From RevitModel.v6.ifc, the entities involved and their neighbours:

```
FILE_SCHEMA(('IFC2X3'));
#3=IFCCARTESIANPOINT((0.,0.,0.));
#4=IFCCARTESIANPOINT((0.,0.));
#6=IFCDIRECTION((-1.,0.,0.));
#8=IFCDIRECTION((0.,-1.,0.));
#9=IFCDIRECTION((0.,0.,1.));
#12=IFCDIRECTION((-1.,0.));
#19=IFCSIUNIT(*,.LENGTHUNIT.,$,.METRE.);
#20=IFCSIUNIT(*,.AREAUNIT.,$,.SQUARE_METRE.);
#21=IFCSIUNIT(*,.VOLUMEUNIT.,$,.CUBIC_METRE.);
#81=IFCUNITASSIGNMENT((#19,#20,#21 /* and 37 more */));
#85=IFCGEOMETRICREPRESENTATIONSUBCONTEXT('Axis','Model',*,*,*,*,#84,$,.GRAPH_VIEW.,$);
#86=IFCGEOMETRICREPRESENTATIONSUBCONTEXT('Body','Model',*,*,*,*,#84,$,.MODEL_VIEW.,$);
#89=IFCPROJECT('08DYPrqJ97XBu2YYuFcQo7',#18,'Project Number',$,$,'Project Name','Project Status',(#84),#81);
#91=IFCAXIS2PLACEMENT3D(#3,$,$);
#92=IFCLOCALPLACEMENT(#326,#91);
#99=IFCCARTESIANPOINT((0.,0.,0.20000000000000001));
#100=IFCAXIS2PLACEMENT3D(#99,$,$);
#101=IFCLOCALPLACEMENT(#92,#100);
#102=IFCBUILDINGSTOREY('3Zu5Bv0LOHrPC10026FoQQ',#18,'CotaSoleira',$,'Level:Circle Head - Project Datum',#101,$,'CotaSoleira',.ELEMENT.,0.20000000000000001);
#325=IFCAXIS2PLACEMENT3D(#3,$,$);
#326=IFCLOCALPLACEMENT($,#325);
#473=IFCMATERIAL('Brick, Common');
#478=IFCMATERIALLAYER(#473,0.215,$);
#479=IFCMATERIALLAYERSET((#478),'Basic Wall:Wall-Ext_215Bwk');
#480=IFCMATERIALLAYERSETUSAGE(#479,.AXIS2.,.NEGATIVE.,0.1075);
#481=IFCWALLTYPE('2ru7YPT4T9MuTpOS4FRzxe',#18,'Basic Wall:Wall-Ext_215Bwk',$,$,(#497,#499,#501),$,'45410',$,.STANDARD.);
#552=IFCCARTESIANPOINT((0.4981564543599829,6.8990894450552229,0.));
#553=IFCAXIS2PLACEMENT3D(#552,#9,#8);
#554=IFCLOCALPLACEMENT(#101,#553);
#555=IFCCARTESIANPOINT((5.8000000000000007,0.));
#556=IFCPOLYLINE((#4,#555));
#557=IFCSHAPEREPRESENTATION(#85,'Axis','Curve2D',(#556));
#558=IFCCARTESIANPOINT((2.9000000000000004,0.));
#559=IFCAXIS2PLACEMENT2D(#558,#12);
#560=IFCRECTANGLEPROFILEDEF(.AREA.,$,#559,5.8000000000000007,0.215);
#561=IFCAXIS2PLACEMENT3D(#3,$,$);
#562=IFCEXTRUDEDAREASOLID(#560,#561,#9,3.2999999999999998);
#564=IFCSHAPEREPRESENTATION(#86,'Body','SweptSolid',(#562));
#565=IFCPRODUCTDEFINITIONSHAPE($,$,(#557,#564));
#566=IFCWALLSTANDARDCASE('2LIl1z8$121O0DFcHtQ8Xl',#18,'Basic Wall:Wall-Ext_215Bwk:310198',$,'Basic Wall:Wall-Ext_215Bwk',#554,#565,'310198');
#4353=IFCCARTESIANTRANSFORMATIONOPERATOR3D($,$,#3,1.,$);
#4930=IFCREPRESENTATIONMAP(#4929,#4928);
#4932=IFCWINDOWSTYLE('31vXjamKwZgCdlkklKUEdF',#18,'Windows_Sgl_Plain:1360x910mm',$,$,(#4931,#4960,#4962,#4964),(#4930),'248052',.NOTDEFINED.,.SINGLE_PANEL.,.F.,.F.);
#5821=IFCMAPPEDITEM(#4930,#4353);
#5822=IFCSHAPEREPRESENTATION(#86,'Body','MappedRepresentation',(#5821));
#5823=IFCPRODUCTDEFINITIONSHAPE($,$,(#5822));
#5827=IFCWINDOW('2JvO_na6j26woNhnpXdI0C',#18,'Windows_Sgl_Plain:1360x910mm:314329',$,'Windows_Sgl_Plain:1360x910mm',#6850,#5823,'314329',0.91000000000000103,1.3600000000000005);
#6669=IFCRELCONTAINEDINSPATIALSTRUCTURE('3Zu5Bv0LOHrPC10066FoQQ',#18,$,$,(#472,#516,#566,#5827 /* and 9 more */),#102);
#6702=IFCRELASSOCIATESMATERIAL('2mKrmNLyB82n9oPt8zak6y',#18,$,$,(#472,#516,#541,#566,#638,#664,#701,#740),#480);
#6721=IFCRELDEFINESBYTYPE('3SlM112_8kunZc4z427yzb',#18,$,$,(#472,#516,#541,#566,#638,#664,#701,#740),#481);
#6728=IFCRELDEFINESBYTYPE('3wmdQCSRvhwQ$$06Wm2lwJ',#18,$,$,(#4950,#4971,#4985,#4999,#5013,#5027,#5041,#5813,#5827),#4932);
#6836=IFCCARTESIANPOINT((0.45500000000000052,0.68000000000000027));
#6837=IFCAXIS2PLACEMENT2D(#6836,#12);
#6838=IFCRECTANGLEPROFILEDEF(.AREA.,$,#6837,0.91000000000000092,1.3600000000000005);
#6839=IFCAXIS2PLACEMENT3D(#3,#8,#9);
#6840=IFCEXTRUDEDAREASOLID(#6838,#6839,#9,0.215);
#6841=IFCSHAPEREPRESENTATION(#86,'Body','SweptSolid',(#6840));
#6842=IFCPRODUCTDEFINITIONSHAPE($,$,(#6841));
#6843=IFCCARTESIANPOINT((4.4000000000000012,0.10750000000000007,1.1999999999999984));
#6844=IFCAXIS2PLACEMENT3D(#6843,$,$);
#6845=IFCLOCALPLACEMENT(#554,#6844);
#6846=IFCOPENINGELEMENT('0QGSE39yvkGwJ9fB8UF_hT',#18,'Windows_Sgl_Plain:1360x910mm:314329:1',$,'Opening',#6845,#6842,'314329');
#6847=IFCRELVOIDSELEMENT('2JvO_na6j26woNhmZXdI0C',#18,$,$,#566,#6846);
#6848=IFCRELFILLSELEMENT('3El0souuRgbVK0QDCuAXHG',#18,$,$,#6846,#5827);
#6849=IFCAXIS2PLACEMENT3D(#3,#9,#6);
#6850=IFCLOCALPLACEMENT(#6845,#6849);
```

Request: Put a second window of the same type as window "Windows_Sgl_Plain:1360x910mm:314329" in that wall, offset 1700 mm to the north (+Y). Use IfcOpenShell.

```python
import ifcopenshell
import ifcopenshell.api.feature
import ifcopenshell.api.geometry
import ifcopenshell.api.root
import ifcopenshell.geom
import ifcopenshell.util.element
import ifcopenshell.util.placement
import ifcopenshell.util.shape

model = ifcopenshell.open("RevitModel.v6.ifc")
settings = ifcopenshell.geom.settings()


def volume(element):
    """Net volume in cubic metres, openings subtracted."""
    shape = ifcopenshell.geom.create_shape(settings, element)
    return ifcopenshell.util.shape.get_volume(shape.geometry)


def reuse_history(source, copy):
    """copy_class also copies each property set's owner history, people and application; keep the originals."""
    for rel in copy.IsDefinedBy:
        if rel.is_a("IfcRelDefinesByProperties") and (history := rel.RelatingPropertyDefinition.OwnerHistory):
            rel.RelatingPropertyDefinition.OwnerHistory = source.OwnerHistory
            ifcopenshell.util.element.remove_deep2(model, history)


window = model.by_id(5827)
opening = window.FillsVoids[0].RelatingOpeningElement
wall = opening.VoidsElements[0].RelatingBuildingElement
before = volume(wall)
shift = ifcopenshell.util.placement.get_local_placement(wall.ObjectPlacement)[:3, 0] * -1.7

# copy_class copies the void relationship, type, container and properties, but no geometry.
new_opening = ifcopenshell.api.root.copy_class(model, product=opening)
new_opening.Representation = ifcopenshell.util.element.copy_deep(
    model, opening.Representation, exclude=["IfcGeometricRepresentationContext", "IfcRepresentationMap"]
)
new_opening.Name = "Windows_Sgl_Plain:1360x910mm"
new_opening.Tag = None
new_window = ifcopenshell.api.root.copy_class(model, product=window)
new_window.Representation = ifcopenshell.util.element.copy_deep(
    model, window.Representation, exclude=["IfcGeometricRepresentationContext", "IfcRepresentationMap"]
)
new_window.Name = "Windows_Sgl_Plain:1360x910mm"
new_window.Tag = None
reuse_history(window, new_window)
fills = ifcopenshell.api.feature.add_filling(model, opening=new_opening, element=new_window)
fills.OwnerHistory = new_window.OwnerHistory  # required in IFC2X3

for old, new in ((opening, new_opening), (window, new_window)):
    matrix = ifcopenshell.util.placement.get_local_placement(old.ObjectPlacement)
    matrix[:3, 3] += shift
    ifcopenshell.api.geometry.edit_object_placement(model, product=new, matrix=matrix, is_si=False)

after = volume(wall)

print(f"wall volume {before:.3f} -> {after:.3f} m3")

model.write("RevitModel.v6_rev.ifc")
```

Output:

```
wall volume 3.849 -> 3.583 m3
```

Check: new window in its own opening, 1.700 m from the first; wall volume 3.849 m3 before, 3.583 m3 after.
